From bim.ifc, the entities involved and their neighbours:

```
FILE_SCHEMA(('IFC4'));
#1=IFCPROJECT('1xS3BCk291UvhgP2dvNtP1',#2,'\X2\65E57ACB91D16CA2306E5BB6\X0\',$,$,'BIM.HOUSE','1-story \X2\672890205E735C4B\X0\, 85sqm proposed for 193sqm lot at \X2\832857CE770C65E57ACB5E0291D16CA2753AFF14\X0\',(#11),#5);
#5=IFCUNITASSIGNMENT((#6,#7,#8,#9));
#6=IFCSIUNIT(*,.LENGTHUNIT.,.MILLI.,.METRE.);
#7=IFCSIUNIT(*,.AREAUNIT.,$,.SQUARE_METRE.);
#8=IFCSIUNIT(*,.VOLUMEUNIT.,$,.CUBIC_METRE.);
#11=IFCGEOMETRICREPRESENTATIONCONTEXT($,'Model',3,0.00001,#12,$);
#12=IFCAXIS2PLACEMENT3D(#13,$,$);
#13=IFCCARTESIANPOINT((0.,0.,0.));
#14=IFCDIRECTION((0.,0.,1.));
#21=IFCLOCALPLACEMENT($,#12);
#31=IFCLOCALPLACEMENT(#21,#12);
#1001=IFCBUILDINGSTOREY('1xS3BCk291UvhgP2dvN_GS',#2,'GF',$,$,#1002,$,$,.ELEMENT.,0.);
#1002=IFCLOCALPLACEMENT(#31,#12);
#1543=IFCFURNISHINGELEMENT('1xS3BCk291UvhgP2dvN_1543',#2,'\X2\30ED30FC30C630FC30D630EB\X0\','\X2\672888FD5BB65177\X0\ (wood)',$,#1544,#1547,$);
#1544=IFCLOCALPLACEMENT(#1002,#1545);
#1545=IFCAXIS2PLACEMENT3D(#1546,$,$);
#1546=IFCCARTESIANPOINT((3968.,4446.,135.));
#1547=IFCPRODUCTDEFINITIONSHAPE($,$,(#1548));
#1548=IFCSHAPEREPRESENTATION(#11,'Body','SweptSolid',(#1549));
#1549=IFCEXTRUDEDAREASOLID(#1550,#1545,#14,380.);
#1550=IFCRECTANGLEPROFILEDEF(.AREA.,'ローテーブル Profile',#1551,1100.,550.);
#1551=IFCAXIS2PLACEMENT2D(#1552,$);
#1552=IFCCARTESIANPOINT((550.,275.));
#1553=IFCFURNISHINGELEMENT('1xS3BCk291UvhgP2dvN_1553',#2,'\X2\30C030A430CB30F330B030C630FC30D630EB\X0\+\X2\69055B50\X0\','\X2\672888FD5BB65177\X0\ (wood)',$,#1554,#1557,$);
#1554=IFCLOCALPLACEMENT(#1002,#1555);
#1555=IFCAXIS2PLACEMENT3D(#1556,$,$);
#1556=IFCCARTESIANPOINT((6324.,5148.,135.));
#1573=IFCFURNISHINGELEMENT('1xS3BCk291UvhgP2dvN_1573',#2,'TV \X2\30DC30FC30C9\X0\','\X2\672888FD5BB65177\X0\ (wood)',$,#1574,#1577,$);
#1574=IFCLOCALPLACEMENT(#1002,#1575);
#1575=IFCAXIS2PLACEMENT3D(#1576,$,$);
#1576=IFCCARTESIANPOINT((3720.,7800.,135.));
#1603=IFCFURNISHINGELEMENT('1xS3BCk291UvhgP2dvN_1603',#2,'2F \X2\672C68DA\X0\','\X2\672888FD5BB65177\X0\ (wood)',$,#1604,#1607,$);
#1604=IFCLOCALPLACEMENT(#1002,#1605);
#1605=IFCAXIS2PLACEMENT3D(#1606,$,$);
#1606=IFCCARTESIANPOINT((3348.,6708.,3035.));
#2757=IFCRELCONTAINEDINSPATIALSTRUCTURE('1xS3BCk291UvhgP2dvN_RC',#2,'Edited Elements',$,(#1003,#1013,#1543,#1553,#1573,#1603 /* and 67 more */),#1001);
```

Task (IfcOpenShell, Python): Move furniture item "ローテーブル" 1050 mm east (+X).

```python
import ifcopenshell
import ifcopenshell.api.geometry
import ifcopenshell.util.placement

model = ifcopenshell.open("bim.ifc")

item = model.by_id(1543)
matrix = ifcopenshell.util.placement.get_local_placement(item.ObjectPlacement)
matrix[0, 3] += 1050.0
ifcopenshell.api.geometry.edit_object_placement(model, product=item, matrix=matrix, is_si=False)

print(ifcopenshell.util.placement.get_local_placement(item.ObjectPlacement).round(3) + 0.0)

model.write("bim_rev.ifc")
```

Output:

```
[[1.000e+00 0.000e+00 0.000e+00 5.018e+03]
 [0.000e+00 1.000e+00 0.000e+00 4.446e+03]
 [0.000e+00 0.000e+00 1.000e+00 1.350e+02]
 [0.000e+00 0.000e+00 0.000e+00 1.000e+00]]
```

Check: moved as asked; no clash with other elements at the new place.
